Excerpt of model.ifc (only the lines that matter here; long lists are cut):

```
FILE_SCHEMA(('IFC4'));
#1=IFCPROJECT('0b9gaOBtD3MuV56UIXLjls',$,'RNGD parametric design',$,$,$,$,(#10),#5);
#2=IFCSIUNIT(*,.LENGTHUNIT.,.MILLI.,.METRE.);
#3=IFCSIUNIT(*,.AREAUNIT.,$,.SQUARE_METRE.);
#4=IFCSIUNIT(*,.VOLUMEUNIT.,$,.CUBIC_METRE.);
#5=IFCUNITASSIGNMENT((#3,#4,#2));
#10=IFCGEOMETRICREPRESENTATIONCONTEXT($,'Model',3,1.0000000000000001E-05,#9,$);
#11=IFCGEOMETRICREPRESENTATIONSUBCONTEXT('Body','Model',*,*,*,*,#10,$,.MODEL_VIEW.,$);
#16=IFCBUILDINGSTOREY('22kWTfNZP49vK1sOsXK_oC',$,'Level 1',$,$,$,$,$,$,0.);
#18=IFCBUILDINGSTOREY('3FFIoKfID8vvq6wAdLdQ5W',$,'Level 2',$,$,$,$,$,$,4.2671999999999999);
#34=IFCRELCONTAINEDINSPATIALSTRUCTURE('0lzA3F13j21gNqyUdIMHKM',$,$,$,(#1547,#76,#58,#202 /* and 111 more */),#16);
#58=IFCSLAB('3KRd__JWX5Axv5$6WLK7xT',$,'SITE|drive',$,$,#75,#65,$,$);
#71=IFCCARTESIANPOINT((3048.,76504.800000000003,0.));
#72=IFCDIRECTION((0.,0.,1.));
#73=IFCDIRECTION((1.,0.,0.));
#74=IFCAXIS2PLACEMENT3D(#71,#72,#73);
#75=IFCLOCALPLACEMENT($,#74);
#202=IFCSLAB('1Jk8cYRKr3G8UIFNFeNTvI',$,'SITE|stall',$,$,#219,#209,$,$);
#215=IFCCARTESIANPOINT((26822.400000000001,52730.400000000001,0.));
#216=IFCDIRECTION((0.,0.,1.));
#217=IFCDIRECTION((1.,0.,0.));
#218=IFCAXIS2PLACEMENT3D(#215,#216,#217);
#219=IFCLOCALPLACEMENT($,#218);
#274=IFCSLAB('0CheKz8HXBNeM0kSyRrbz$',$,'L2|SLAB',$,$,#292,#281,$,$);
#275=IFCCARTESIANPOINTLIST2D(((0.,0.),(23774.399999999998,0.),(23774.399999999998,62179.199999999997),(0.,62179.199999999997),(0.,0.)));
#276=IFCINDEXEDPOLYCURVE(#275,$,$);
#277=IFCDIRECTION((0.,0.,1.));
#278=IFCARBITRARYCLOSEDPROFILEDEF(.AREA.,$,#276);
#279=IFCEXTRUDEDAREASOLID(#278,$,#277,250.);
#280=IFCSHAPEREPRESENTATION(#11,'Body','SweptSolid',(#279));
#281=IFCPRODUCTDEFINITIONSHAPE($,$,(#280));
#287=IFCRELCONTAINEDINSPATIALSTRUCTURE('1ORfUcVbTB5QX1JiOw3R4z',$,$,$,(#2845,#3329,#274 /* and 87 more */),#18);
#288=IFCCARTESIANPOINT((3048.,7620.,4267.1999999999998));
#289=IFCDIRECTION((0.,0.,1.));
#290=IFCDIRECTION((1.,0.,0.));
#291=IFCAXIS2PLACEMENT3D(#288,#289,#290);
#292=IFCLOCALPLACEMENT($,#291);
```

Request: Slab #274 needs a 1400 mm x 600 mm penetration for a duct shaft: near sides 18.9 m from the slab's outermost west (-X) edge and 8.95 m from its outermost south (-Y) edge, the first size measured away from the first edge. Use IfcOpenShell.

```python
import numpy as np
import ifcopenshell
import ifcopenshell.api.feature
import ifcopenshell.api.geometry
import ifcopenshell.api.root
import ifcopenshell.geom
import ifcopenshell.util.placement
import ifcopenshell.util.representation
import ifcopenshell.util.shape
import ifcopenshell.util.unit

model = ifcopenshell.open("model.ifc")
unit_scale = ifcopenshell.util.unit.calculate_unit_scale(model)
settings = ifcopenshell.geom.settings()


def volume(element):
    """Net volume in cubic metres, openings subtracted."""
    shape = ifcopenshell.geom.create_shape(settings, element)
    return ifcopenshell.util.shape.get_volume(shape.geometry)


slab = model.by_id(274)
before = volume(slab)

# Extent in the slab's own axes, in metres. The edges named are its -X and -Y sides.
slab_shape = ifcopenshell.geom.create_shape(settings, slab)
vertices = ifcopenshell.util.shape.get_vertices(slab_shape.geometry)
x_min, y_min, bottom = vertices.min(axis=0)
top = vertices[:, 2].max()

opening = ifcopenshell.api.root.create_entity(model, ifc_class="IfcOpeningElement", name="Duct shaft opening", predefined_type="OPENING")
context = ifcopenshell.util.representation.get_context(model, "Model", "Body", "MODEL_VIEW")
width, depth = 1.4, 0.6
outline = [(0.0, 0.0), (width, 0.0), (width, depth), (0.0, depth), (0.0, 0.0)]
# Overshoot both faces by 50 mm so the cut is clean.
shape = ifcopenshell.api.geometry.add_slab_representation(
    model, context=context, depth=top - bottom + 0.1, polyline=outline
)
ifcopenshell.api.geometry.assign_representation(model, product=opening, representation=shape)

matrix = ifcopenshell.util.placement.get_local_placement(slab.ObjectPlacement)
matrix[:, 3] = matrix @ np.append(np.array([x_min + 18.9, y_min + 8.95, bottom - 0.05]) / unit_scale, 1.0)
ifcopenshell.api.geometry.edit_object_placement(model, product=opening, matrix=matrix, is_si=False)
ifcopenshell.api.feature.add_feature(model, feature=opening, element=slab)

after = volume(slab)

print(f"slab volume {before:.3f} -> {after:.3f} m3")

model.write("model_edited.ifc")
```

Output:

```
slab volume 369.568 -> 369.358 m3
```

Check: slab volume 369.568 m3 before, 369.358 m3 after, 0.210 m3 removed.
